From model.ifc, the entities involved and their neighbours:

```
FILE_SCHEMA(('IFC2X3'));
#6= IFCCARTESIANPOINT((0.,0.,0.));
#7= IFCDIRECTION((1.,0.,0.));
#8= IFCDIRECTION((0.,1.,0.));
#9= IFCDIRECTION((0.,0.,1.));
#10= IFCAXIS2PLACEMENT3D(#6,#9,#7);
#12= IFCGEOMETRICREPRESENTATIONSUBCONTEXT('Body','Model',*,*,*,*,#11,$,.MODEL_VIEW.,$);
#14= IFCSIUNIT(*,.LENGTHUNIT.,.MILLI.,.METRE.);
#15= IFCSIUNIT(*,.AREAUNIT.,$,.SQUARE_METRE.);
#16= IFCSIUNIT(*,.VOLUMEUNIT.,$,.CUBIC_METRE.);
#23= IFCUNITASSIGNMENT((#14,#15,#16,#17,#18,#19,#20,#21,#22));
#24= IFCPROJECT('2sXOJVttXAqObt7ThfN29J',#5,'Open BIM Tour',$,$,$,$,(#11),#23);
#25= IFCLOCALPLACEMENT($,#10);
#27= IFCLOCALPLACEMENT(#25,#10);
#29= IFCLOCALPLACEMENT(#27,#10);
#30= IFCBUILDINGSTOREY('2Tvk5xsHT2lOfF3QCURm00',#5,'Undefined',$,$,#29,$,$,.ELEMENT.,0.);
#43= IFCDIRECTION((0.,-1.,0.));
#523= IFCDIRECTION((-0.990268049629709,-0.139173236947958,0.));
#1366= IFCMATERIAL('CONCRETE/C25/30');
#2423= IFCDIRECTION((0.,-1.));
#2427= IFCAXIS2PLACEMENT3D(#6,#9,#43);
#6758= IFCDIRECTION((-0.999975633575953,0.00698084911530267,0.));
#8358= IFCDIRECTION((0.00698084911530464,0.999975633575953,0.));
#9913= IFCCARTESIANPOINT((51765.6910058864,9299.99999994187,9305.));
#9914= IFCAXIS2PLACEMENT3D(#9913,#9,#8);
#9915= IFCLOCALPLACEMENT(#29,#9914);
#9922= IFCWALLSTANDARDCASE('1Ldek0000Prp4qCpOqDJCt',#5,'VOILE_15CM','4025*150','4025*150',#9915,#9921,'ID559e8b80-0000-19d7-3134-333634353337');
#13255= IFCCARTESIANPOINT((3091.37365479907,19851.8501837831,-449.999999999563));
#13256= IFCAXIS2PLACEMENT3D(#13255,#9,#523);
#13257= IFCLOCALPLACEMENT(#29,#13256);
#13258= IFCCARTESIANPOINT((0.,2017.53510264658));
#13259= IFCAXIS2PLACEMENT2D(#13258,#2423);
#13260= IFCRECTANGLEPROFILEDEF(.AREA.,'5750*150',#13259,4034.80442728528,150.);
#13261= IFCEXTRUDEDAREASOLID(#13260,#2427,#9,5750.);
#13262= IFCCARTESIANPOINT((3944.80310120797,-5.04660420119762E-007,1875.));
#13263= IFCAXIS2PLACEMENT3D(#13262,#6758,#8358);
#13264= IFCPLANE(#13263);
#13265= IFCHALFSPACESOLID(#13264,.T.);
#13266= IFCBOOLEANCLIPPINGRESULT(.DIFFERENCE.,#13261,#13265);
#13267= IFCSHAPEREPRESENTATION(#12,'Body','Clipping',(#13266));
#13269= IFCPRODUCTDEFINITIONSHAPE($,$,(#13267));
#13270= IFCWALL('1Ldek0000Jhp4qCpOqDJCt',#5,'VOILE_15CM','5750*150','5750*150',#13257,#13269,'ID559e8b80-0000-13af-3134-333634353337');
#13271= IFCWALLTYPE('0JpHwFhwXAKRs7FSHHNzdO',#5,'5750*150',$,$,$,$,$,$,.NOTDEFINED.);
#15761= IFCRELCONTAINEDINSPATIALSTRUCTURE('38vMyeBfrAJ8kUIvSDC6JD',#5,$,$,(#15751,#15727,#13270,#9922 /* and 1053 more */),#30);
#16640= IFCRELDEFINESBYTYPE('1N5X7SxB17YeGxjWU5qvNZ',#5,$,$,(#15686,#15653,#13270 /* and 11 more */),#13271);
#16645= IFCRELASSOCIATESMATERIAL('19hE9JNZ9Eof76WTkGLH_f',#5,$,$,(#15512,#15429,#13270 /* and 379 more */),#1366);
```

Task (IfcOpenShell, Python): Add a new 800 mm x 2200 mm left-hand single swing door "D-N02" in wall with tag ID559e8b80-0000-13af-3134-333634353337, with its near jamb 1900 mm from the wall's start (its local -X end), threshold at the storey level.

```python
import numpy as np
import ifcopenshell
import ifcopenshell.api.feature
import ifcopenshell.api.geometry
import ifcopenshell.api.root
import ifcopenshell.api.spatial
import ifcopenshell.api.type
import ifcopenshell.geom
import ifcopenshell.util.element
import ifcopenshell.util.placement
import ifcopenshell.util.representation
import ifcopenshell.util.shape
import ifcopenshell.util.unit

model = ifcopenshell.open("model.ifc")
unit_scale = ifcopenshell.util.unit.calculate_unit_scale(model)
settings = ifcopenshell.geom.settings()


def volume(element):
    """Net volume in cubic metres, openings subtracted."""
    shape = ifcopenshell.geom.create_shape(settings, element)
    return ifcopenshell.util.shape.get_volume(shape.geometry)


wall = model.by_id(13270)
storey = ifcopenshell.util.element.get_container(wall, ifc_class="IfcBuildingStorey")
context = ifcopenshell.util.representation.get_context(model, "Model", "Body", "MODEL_VIEW")
before = volume(wall)

width, height, from_end, sill = 0.8, 2.2, 1.9, 0.0  # metres

# The wall runs along its own X axis, and the end named is its -X end.
wall_shape = ifcopenshell.geom.create_shape(settings, wall)
x, y, z = ifcopenshell.util.shape.get_vertices(wall_shape.geometry).T
start = x.min() + from_end
face, thickness = float(y.min()), float(y.max() - y.min())
wall_matrix = ifcopenshell.util.placement.get_local_placement(wall.ObjectPlacement)
level = ifcopenshell.util.placement.get_local_placement(storey.ObjectPlacement)[2, 3]


def in_wall(x, y):
    """Placement at x, y metres in the wall's axes, at sill height."""
    matrix = wall_matrix.copy()
    matrix[:, 3] = wall_matrix @ np.array([x / unit_scale, y / unit_scale, 0.0, 1.0])
    matrix[2, 3] = level + sill / unit_scale
    return matrix


# Opening: a box that overshoots both wall faces by 50 mm.
opening = ifcopenshell.api.root.create_entity(model, ifc_class="IfcOpeningElement")
box = ifcopenshell.api.geometry.add_wall_representation(
    model, context=context, length=width, height=height, thickness=thickness + 0.1
)
ifcopenshell.api.geometry.assign_representation(model, product=opening, representation=box)
ifcopenshell.api.geometry.edit_object_placement(model, product=opening, matrix=in_wall(start, face - 0.05), is_si=False)
ifcopenshell.api.feature.add_feature(model, feature=opening, element=wall)

door = ifcopenshell.api.root.create_entity(model, ifc_class="IfcDoor", name="D-N02")
door.OverallWidth, door.OverallHeight = width / unit_scale, height / unit_scale
body = ifcopenshell.api.geometry.add_door_representation(
    model,
    context=context,
    overall_width=door.OverallWidth,
    overall_height=door.OverallHeight,
    operation_type="SINGLE_SWING_LEFT",
    lining_properties={"LiningDepth": thickness / unit_scale, "ThresholdDepth": thickness / unit_scale},
)
ifcopenshell.api.geometry.assign_representation(model, product=door, representation=body)
ifcopenshell.api.spatial.assign_container(model, products=[door], relating_structure=storey)
fills = ifcopenshell.api.feature.add_filling(model, opening=opening, element=door)
fills.OwnerHistory = door.OwnerHistory  # required in IFC2X3

# IFC2X3 keeps the operation on the door style.
style = ifcopenshell.api.root.create_entity(model, ifc_class="IfcDoorStyle", name="D-N02")
style.OperationType, style.ConstructionType = "SINGLE_SWING_LEFT", "NOTDEFINED"
style.ParameterTakesPrecedence = style.Sizeable = False
ifcopenshell.api.type.assign_type(model, related_objects=[door], relating_type=style)

# The lining spans the wall, so the door starts at the wall face.
ifcopenshell.api.geometry.edit_object_placement(model, product=door, matrix=in_wall(start, face), is_si=False)

after = volume(wall)

print(f"wall volume {before:.3f} -> {after:.3f} m3")

model.write("model-out.ifc")
```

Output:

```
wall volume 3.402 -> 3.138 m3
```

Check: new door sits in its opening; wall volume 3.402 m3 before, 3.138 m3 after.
